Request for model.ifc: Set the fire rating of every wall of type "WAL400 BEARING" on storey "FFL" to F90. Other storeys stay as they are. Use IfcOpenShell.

First a look at what the model holds.

```python
import ifcopenshell
import ifcopenshell.util.element

model = ifcopenshell.open("model.ifc")
print(model.schema)
storey = next(s for s in model.by_type("IfcBuildingStorey") if s.Name == "FFL")
walls = [e for e in ifcopenshell.util.element.get_decomposition(storey) if e.is_a("IfcWall")]
seen = {}
for e in walls:
    element_type = ifcopenshell.util.element.get_type(e)
    key = (element_type.Name if element_type != e and element_type else None, ifcopenshell.util.element.get_pset(e, "Pset_WallCommon", "FireRating"))
    seen[key] = seen.get(key, 0) + 1
for (name, value), count in sorted(seen.items(), key=str):
    print(count, "x", name, "|", value)
```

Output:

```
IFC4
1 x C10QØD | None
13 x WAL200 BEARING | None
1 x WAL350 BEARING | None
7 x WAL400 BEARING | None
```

```python
import ifcopenshell
import ifcopenshell.api.pset
import ifcopenshell.util.element

model = ifcopenshell.open("model.ifc")

storey = next(s for s in model.by_type("IfcBuildingStorey") if s.Name == "FFL")
walls = [e for e in ifcopenshell.util.element.get_decomposition(storey) if e.is_a("IfcWall")]

count = 0
for e in walls:
    element_type = ifcopenshell.util.element.get_type(e)
    if element_type in (None, e) or element_type.Name != "WAL400 BEARING":
        continue
    # add_pset returns the element's existing set when there is one.
    pset = ifcopenshell.api.pset.add_pset(model, product=e, name="Pset_WallCommon")
    ifcopenshell.api.pset.edit_pset(model, pset=pset, properties={"FireRating": "F90"})
    count += 1

print(count, "walls updated")

model.write("model_edited.ifc")
```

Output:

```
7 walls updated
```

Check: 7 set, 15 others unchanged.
